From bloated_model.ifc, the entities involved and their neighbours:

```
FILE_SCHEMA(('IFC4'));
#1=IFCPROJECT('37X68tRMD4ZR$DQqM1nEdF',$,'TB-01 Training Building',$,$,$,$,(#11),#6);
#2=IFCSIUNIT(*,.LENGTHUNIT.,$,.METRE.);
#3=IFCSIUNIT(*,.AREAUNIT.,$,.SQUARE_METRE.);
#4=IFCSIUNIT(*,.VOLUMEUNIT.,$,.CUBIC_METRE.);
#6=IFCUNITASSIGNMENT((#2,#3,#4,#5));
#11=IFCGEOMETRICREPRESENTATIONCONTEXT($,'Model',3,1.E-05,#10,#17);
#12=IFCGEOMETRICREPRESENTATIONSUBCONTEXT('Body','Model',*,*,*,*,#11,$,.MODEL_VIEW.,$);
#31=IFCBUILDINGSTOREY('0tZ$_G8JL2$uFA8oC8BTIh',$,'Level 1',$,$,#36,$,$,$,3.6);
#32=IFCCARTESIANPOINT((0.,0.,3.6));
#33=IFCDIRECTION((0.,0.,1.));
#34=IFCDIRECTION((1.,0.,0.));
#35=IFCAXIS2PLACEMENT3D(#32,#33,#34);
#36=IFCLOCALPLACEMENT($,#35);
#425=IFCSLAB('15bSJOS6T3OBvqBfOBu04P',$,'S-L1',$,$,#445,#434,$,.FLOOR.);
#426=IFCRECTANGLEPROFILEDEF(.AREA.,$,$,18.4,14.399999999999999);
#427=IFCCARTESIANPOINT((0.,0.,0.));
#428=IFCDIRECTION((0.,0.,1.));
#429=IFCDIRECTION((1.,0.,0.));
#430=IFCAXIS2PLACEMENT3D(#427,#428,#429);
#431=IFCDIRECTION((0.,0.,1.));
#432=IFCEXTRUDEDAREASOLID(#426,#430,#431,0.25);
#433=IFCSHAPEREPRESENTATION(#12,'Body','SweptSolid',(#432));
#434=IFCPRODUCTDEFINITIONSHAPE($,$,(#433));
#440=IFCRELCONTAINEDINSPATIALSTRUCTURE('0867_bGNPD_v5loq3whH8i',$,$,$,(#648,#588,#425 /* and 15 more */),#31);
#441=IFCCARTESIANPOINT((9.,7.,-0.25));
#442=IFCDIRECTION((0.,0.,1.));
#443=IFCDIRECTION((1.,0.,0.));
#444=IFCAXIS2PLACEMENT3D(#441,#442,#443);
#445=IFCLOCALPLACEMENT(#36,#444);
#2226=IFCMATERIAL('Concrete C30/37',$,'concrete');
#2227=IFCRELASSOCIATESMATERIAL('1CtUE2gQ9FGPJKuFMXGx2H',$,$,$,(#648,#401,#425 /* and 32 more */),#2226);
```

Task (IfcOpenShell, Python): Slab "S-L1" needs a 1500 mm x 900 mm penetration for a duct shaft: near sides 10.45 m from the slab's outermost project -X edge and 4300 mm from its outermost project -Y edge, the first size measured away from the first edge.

```python
import numpy as np
import ifcopenshell
import ifcopenshell.api.feature
import ifcopenshell.api.geometry
import ifcopenshell.api.root
import ifcopenshell.geom
import ifcopenshell.util.placement
import ifcopenshell.util.representation
import ifcopenshell.util.shape
import ifcopenshell.util.unit

model = ifcopenshell.open("bloated_model.ifc")
unit_scale = ifcopenshell.util.unit.calculate_unit_scale(model)
settings = ifcopenshell.geom.settings()


def volume(element):
    """Net volume in cubic metres, openings subtracted."""
    shape = ifcopenshell.geom.create_shape(settings, element)
    return ifcopenshell.util.shape.get_volume(shape.geometry)


slab = model.by_id(425)
before = volume(slab)

# Extent in the slab's own axes, in metres. The edges named are its -X and -Y sides.
slab_shape = ifcopenshell.geom.create_shape(settings, slab)
vertices = ifcopenshell.util.shape.get_vertices(slab_shape.geometry)
x_min, y_min, bottom = vertices.min(axis=0)
top = vertices[:, 2].max()

opening = ifcopenshell.api.root.create_entity(model, ifc_class="IfcOpeningElement", name="Duct shaft opening", predefined_type="OPENING")
context = ifcopenshell.util.representation.get_context(model, "Model", "Body", "MODEL_VIEW")
width, depth = 1.5, 0.9
outline = [(0.0, 0.0), (width, 0.0), (width, depth), (0.0, depth), (0.0, 0.0)]
# Overshoot both faces by 50 mm so the cut is clean.
shape = ifcopenshell.api.geometry.add_slab_representation(
    model, context=context, depth=top - bottom + 0.1, polyline=outline
)
ifcopenshell.api.geometry.assign_representation(model, product=opening, representation=shape)

matrix = ifcopenshell.util.placement.get_local_placement(slab.ObjectPlacement)
matrix[:, 3] = matrix @ np.append(np.array([x_min + 10.45, y_min + 4.3, bottom - 0.05]) / unit_scale, 1.0)
ifcopenshell.api.geometry.edit_object_placement(model, product=opening, matrix=matrix, is_si=False)
ifcopenshell.api.feature.add_feature(model, feature=opening, element=slab)

after = volume(slab)

print(f"slab volume {before:.3f} -> {after:.3f} m3")

model.write("bloated_model_v2.ifc")
```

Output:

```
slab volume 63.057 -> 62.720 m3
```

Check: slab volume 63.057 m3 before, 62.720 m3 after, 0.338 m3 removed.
